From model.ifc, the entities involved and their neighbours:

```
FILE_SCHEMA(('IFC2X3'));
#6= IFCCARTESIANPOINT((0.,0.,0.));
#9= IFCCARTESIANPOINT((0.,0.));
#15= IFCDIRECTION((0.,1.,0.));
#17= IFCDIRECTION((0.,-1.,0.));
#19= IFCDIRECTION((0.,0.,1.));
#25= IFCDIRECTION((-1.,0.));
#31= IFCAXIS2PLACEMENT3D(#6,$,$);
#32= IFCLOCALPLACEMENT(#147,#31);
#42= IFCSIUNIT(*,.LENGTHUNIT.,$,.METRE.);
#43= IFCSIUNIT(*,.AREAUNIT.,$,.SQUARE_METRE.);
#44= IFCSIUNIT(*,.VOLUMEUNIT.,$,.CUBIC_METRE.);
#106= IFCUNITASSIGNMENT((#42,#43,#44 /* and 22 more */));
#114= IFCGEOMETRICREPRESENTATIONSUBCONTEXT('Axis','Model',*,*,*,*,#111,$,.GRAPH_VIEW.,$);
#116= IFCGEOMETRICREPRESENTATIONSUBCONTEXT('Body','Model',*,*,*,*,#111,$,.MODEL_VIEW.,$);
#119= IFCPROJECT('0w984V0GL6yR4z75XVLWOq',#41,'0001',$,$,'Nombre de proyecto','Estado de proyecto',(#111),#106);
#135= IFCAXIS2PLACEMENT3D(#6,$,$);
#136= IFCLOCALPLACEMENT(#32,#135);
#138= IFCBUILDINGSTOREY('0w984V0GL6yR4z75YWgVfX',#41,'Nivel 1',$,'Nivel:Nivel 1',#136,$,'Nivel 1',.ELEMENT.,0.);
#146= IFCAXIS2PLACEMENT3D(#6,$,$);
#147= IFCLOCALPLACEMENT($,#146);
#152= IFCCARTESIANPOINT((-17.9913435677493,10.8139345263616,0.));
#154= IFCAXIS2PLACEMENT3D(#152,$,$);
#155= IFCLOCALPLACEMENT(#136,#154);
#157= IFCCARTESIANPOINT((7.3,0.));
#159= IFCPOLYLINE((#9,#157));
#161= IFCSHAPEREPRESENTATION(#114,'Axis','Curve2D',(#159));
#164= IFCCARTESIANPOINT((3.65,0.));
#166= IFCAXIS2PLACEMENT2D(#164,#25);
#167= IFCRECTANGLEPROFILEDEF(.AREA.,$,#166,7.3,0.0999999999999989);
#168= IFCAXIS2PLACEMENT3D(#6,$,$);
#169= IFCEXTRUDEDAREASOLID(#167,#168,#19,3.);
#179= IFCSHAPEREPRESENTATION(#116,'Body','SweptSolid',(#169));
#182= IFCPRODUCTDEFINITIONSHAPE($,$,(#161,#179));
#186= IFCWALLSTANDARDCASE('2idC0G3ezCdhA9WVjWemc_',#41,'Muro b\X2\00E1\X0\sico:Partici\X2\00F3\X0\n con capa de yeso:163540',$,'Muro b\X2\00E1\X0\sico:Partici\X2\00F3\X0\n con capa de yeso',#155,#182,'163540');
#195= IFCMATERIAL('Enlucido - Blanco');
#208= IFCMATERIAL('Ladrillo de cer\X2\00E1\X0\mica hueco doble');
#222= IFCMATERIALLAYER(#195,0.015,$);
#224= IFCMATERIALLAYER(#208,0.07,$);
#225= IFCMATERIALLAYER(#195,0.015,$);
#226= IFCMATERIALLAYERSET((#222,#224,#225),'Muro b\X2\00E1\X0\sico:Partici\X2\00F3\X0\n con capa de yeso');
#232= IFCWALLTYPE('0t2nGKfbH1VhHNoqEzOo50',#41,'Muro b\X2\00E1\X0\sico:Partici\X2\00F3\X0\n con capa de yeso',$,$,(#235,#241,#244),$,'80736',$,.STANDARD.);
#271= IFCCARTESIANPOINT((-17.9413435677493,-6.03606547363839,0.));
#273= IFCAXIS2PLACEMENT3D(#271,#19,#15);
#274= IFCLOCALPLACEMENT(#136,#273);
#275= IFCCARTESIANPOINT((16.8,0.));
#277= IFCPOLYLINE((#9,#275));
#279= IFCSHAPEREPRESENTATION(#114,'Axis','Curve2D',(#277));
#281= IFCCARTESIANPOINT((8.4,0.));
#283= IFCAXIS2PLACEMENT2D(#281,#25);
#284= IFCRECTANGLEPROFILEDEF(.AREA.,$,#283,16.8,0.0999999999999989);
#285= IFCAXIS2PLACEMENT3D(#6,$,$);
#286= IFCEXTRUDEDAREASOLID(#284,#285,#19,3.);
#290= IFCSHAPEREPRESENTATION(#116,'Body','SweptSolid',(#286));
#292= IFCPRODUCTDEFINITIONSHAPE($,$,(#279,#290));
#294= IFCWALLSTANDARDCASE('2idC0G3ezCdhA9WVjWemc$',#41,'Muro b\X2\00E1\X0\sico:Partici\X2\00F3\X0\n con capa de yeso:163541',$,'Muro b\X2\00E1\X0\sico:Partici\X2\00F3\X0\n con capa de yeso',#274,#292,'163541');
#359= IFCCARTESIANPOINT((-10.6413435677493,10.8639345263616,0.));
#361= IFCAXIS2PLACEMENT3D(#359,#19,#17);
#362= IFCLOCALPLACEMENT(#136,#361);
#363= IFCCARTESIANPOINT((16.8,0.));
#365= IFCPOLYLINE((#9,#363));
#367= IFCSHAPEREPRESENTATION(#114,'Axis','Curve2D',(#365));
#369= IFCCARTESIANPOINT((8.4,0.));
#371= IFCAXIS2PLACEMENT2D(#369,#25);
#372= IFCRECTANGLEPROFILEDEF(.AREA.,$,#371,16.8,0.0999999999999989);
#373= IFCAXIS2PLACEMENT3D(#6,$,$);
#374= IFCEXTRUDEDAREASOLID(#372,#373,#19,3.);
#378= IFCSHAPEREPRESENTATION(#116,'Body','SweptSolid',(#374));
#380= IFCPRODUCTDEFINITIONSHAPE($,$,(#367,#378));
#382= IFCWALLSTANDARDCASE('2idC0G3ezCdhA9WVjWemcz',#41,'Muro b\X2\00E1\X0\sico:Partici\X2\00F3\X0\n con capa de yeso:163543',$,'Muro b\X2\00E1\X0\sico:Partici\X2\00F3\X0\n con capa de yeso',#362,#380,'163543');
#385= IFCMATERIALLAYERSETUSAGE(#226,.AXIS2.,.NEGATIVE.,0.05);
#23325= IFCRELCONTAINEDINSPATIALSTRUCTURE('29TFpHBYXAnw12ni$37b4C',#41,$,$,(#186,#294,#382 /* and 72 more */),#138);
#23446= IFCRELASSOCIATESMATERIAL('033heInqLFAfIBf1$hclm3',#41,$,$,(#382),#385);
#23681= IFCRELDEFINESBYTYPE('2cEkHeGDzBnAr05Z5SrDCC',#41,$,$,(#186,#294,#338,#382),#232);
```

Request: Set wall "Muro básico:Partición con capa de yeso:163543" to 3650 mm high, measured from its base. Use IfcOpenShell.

```python
import ifcopenshell
import ifcopenshell.geom
import ifcopenshell.util.representation
import ifcopenshell.util.shape
import ifcopenshell.util.unit

model = ifcopenshell.open("model.ifc")
unit_scale = ifcopenshell.util.unit.calculate_unit_scale(model)
settings = ifcopenshell.geom.settings()


def volume(element):
    """Net volume in cubic metres, openings subtracted."""
    shape = ifcopenshell.geom.create_shape(settings, element)
    return ifcopenshell.util.shape.get_volume(shape.geometry)


wall = model.by_id(382)
before = volume(wall)

body = ifcopenshell.util.representation.get_representation(wall, "Model", "Body")
solid = body.Items[0]
old_height = solid.Depth
solid.Depth = 3.65 / unit_scale
after = volume(wall)

print(f"height {old_height:g} -> {solid.Depth:g}, volume {before:.3f} -> {after:.3f} m3")

model.write("model_rev.ifc")
```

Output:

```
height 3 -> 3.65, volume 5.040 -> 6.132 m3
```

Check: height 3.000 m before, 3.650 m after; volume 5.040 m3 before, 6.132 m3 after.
